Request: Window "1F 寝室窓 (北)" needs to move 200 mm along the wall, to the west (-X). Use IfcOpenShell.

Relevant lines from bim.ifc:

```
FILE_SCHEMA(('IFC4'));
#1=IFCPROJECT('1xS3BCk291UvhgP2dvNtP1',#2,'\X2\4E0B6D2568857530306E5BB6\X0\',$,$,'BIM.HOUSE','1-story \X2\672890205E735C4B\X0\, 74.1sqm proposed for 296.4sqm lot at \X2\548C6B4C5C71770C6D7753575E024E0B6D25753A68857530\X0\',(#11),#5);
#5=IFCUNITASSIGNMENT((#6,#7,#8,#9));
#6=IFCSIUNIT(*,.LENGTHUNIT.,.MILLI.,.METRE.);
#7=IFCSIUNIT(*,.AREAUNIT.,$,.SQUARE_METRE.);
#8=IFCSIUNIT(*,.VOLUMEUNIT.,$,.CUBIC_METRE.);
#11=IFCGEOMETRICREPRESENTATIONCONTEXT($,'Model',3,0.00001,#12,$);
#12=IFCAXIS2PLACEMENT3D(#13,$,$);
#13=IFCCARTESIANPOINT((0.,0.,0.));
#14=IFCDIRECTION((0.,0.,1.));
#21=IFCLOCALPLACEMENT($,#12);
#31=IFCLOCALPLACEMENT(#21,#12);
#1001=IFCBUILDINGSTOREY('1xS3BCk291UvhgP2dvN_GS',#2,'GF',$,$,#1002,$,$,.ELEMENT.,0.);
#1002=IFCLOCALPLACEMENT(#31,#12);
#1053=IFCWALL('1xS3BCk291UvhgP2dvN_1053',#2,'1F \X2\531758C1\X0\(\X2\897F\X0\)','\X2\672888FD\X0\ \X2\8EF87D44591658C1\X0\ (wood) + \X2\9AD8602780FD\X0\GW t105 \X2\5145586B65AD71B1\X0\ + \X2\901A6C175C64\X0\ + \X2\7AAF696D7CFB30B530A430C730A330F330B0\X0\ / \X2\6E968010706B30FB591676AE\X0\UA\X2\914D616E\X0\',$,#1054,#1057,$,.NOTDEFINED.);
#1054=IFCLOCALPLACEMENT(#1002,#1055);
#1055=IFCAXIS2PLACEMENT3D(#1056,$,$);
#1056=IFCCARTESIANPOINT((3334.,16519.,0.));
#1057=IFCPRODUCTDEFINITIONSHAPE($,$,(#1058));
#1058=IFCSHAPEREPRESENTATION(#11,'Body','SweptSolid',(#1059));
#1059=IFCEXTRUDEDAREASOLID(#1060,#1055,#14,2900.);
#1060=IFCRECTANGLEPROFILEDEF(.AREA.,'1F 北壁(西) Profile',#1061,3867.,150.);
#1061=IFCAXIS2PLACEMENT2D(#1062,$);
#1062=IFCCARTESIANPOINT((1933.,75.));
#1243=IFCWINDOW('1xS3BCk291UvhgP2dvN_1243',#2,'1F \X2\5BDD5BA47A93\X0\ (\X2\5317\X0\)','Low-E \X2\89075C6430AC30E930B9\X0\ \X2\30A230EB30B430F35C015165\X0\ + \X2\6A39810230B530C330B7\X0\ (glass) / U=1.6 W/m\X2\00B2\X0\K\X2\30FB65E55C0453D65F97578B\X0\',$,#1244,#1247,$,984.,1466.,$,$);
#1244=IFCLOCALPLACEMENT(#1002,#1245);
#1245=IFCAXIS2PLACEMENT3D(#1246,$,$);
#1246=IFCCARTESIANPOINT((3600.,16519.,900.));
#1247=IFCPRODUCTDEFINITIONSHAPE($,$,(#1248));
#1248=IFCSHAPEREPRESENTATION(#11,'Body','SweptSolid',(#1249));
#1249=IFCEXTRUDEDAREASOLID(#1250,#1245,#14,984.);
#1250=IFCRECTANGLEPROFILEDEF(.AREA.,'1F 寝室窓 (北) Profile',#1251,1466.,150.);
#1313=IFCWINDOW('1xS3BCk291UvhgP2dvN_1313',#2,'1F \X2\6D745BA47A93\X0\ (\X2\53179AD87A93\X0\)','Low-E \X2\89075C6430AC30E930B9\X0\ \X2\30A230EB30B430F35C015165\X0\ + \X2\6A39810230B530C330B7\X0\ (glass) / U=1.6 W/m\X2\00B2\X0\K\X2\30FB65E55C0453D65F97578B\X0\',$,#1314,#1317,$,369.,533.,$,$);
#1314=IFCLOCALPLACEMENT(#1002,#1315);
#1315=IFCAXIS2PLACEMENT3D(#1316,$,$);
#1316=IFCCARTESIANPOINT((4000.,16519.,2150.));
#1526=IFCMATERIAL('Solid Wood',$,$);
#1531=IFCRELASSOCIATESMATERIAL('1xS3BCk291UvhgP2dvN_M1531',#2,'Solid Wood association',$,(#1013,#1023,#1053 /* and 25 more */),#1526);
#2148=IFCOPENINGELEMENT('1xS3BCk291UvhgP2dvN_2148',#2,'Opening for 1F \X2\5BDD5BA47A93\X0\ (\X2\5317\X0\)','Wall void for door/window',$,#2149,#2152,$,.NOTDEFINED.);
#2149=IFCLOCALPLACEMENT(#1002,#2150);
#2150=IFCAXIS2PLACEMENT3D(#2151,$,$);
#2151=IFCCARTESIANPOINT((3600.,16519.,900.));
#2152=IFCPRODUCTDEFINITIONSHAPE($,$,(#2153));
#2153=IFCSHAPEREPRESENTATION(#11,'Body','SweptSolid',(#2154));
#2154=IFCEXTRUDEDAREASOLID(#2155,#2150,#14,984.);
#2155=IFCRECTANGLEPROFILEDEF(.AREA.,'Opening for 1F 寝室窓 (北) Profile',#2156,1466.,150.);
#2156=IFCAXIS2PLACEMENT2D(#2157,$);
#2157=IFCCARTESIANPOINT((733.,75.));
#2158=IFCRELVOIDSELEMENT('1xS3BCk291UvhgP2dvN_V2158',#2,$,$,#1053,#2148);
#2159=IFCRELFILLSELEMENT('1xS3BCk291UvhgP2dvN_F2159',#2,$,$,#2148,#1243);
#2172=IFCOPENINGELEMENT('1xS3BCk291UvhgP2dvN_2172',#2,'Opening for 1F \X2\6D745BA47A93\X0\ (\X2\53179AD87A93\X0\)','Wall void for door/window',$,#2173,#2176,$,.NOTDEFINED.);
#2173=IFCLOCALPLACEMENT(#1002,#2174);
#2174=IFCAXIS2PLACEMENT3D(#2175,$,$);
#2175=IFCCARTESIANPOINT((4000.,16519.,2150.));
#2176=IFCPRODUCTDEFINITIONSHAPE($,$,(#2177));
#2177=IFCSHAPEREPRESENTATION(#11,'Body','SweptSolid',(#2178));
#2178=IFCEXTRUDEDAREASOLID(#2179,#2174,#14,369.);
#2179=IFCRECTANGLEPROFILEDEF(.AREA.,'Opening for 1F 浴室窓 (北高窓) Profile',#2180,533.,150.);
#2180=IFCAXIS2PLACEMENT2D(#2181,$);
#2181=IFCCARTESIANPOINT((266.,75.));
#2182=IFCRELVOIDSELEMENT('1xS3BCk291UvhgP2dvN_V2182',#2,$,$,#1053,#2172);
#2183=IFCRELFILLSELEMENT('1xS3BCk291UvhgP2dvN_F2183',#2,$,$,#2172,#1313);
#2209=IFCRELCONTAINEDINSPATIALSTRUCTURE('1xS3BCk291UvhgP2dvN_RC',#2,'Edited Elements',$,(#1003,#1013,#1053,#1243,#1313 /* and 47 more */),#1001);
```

```python
import ifcopenshell
import ifcopenshell.api.geometry
import ifcopenshell.util.placement
import ifcopenshell.util.unit

model = ifcopenshell.open("bim.ifc")
unit_scale = ifcopenshell.util.unit.calculate_unit_scale(model)

window = model.by_id(1243)
opening = window.FillsVoids[0].RelatingOpeningElement
wall = opening.VoidsElements[0].RelatingBuildingElement

wall_matrix = ifcopenshell.util.placement.get_local_placement(wall.ObjectPlacement)
shift = wall_matrix[:3, 0] * -0.2 / unit_scale
before = ifcopenshell.util.placement.get_local_placement(window.ObjectPlacement)[:3, 3].copy()

# The window is not placed relative to its opening, so move both.
for product in (opening, window):
    matrix = ifcopenshell.util.placement.get_local_placement(product.ObjectPlacement)
    matrix[:3, 3] += shift
    ifcopenshell.api.geometry.edit_object_placement(model, product=product, matrix=matrix, is_si=False)

after = ifcopenshell.util.placement.get_local_placement(window.ObjectPlacement)[:3, 3]
print("window moved by", (after - before).round(3) + 0.0)

model.write("bim_v2.ifc")
```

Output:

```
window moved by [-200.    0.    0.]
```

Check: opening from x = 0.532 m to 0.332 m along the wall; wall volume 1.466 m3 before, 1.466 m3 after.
